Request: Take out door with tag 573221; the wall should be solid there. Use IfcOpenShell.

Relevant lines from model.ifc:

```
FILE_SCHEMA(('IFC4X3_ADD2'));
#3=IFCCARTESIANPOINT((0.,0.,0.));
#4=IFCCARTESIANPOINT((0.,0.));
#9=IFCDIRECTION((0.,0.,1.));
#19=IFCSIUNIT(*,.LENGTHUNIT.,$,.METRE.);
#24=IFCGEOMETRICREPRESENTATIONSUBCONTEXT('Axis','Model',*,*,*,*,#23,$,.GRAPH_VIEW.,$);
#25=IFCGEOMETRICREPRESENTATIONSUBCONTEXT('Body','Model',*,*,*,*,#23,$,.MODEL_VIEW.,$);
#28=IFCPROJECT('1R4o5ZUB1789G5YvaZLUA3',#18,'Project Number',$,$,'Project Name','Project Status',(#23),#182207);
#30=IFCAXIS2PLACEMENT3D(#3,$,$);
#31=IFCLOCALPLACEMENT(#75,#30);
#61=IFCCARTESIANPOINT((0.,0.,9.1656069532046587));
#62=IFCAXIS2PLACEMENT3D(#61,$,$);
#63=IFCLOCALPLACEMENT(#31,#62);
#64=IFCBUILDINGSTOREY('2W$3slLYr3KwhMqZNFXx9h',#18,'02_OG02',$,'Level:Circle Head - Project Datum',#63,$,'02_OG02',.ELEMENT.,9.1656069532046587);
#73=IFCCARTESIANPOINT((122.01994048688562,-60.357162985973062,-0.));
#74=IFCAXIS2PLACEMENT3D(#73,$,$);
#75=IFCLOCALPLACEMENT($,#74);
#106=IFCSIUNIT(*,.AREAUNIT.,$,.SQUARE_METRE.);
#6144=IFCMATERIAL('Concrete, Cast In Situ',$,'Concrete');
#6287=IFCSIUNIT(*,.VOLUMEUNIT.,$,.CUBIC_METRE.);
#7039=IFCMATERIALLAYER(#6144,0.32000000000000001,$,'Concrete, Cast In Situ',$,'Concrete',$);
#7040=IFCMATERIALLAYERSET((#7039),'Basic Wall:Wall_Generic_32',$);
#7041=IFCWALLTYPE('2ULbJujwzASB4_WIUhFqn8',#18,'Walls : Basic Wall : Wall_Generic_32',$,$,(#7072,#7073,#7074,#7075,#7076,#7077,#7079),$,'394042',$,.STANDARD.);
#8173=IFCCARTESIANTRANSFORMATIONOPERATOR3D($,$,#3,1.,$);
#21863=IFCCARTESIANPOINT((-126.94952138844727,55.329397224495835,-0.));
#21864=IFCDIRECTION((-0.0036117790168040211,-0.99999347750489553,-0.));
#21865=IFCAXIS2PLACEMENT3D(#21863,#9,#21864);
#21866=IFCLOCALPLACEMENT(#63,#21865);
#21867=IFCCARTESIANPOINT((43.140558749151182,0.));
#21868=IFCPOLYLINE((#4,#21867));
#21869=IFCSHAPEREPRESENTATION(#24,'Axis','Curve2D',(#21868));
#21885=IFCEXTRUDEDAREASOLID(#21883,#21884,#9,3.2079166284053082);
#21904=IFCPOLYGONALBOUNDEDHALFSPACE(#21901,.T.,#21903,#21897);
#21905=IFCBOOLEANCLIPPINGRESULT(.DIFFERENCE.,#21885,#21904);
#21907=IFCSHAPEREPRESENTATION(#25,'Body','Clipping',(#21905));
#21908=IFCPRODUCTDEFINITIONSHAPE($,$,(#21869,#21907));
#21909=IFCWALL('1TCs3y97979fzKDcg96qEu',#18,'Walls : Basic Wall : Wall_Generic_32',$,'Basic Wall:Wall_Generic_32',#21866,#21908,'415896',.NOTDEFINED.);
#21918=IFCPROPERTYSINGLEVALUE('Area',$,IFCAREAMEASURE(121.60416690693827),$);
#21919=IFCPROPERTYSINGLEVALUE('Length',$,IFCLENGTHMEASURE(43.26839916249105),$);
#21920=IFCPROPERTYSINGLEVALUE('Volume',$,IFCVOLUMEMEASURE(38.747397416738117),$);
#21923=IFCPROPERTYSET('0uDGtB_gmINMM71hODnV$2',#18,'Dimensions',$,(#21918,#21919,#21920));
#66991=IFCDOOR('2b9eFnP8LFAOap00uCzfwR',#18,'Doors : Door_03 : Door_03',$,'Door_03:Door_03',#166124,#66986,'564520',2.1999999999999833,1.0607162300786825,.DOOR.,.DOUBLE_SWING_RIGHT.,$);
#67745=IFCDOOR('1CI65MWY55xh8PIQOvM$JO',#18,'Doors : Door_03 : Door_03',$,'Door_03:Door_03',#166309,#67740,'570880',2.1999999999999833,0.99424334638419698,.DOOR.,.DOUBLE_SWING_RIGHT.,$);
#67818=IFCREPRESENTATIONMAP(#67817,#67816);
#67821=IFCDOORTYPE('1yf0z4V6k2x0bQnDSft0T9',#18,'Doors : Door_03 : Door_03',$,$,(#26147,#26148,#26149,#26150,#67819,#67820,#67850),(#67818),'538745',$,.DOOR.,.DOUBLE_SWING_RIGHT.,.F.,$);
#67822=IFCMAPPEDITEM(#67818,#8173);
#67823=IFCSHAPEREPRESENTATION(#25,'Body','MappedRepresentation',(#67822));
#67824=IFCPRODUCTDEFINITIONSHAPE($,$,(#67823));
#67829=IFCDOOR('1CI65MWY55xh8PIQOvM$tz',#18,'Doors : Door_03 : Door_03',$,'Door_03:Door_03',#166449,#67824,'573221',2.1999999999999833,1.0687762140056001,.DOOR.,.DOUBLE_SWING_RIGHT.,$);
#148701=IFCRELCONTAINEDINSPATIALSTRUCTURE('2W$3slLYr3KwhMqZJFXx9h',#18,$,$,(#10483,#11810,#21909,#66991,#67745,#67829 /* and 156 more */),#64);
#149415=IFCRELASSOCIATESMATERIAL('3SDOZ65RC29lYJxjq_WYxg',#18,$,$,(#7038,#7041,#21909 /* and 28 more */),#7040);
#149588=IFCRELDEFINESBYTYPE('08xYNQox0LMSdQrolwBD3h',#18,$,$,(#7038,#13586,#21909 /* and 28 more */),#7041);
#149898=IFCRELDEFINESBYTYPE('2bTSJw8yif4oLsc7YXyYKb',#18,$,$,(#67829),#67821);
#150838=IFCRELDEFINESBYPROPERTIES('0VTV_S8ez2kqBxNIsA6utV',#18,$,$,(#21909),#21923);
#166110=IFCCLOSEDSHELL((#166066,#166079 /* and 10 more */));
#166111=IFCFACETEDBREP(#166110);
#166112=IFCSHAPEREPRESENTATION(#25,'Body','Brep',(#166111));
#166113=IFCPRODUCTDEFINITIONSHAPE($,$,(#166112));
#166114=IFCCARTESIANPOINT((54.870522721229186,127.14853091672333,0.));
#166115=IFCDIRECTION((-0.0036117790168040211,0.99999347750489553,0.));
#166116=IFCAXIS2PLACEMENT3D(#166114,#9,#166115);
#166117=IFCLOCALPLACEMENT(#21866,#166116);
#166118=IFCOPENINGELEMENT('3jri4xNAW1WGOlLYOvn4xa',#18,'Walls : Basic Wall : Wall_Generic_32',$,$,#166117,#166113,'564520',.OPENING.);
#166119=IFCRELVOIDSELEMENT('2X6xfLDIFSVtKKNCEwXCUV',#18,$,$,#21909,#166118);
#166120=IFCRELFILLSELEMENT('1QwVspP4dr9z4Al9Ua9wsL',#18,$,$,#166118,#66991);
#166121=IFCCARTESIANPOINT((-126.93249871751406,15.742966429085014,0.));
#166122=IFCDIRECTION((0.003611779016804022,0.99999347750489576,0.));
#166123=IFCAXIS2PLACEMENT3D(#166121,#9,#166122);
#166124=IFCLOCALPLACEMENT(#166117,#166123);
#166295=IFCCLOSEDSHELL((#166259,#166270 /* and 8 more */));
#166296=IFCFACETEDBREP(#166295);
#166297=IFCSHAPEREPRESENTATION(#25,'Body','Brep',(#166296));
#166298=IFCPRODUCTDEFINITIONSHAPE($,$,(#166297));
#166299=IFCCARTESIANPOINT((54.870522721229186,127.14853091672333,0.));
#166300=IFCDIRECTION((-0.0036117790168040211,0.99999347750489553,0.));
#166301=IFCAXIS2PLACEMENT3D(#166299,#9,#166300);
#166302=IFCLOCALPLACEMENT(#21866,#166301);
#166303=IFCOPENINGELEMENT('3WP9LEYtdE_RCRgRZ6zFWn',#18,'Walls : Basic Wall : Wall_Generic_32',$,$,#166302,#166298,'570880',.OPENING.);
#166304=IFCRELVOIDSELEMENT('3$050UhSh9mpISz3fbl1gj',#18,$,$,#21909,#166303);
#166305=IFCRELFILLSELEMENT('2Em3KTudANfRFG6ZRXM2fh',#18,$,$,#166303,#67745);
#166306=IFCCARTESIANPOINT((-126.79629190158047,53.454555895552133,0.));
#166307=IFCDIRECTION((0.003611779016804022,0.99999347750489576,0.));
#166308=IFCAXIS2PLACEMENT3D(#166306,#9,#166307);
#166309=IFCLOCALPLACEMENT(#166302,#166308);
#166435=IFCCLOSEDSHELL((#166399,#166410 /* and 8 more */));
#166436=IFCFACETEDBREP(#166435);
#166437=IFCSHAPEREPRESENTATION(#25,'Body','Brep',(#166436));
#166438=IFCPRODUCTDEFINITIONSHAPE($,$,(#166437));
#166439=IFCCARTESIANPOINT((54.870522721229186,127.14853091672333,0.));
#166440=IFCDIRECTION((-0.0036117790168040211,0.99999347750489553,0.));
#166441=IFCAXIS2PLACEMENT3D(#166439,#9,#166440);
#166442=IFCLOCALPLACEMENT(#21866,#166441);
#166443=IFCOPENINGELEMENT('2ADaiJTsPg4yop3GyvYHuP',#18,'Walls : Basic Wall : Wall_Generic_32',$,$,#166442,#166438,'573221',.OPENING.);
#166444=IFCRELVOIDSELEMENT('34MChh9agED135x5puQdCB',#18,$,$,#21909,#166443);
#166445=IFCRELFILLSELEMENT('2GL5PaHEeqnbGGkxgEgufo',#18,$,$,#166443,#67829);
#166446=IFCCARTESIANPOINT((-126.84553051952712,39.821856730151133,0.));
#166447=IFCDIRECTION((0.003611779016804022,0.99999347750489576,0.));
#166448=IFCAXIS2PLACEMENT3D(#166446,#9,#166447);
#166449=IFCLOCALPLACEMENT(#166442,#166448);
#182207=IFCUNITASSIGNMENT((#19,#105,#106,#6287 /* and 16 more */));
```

```python
import ifcopenshell
import ifcopenshell.api.feature
import ifcopenshell.api.pset
import ifcopenshell.api.root
import ifcopenshell.geom
import ifcopenshell.util.element
import ifcopenshell.util.shape
import ifcopenshell.util.unit

model = ifcopenshell.open("model.ifc")
area_scale = ifcopenshell.util.unit.calculate_unit_scale(model, "AREAUNIT")
volume_scale = ifcopenshell.util.unit.calculate_unit_scale(model, "VOLUMEUNIT")
settings = ifcopenshell.geom.settings()


def volume(element):
    """Net volume in cubic metres, openings subtracted."""
    shape = ifcopenshell.geom.create_shape(settings, element)
    return ifcopenshell.util.shape.get_volume(shape.geometry)


door = model.by_guid("1CI65MWY55xh8PIQOvM$tz")
opening = door.FillsVoids[0].RelatingOpeningElement
wall = opening.VoidsElements[0].RelatingBuildingElement
before = volume(wall)

ifcopenshell.api.root.remove_product(model, product=door)
ifcopenshell.api.feature.remove_feature(model, feature=opening)

after = volume(wall)
thickness = 0.32  # wall thickness in metres

# Update the wall's stored quantities.
pset = model.by_id(ifcopenshell.util.element.get_pset(wall, "Dimensions", should_inherit=False)["id"])
ifcopenshell.api.pset.edit_pset(model, pset=pset, properties={
    "Area": model.create_entity("IfcAreaMeasure", after / thickness / area_scale),
    "Volume": model.create_entity("IfcVolumeMeasure", after / volume_scale),
})

print(f"wall volume {before:.3f} -> {after:.3f} m3")

model.write("model_rev.ifc")
```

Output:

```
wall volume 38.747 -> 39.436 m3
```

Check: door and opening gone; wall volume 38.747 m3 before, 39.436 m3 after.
